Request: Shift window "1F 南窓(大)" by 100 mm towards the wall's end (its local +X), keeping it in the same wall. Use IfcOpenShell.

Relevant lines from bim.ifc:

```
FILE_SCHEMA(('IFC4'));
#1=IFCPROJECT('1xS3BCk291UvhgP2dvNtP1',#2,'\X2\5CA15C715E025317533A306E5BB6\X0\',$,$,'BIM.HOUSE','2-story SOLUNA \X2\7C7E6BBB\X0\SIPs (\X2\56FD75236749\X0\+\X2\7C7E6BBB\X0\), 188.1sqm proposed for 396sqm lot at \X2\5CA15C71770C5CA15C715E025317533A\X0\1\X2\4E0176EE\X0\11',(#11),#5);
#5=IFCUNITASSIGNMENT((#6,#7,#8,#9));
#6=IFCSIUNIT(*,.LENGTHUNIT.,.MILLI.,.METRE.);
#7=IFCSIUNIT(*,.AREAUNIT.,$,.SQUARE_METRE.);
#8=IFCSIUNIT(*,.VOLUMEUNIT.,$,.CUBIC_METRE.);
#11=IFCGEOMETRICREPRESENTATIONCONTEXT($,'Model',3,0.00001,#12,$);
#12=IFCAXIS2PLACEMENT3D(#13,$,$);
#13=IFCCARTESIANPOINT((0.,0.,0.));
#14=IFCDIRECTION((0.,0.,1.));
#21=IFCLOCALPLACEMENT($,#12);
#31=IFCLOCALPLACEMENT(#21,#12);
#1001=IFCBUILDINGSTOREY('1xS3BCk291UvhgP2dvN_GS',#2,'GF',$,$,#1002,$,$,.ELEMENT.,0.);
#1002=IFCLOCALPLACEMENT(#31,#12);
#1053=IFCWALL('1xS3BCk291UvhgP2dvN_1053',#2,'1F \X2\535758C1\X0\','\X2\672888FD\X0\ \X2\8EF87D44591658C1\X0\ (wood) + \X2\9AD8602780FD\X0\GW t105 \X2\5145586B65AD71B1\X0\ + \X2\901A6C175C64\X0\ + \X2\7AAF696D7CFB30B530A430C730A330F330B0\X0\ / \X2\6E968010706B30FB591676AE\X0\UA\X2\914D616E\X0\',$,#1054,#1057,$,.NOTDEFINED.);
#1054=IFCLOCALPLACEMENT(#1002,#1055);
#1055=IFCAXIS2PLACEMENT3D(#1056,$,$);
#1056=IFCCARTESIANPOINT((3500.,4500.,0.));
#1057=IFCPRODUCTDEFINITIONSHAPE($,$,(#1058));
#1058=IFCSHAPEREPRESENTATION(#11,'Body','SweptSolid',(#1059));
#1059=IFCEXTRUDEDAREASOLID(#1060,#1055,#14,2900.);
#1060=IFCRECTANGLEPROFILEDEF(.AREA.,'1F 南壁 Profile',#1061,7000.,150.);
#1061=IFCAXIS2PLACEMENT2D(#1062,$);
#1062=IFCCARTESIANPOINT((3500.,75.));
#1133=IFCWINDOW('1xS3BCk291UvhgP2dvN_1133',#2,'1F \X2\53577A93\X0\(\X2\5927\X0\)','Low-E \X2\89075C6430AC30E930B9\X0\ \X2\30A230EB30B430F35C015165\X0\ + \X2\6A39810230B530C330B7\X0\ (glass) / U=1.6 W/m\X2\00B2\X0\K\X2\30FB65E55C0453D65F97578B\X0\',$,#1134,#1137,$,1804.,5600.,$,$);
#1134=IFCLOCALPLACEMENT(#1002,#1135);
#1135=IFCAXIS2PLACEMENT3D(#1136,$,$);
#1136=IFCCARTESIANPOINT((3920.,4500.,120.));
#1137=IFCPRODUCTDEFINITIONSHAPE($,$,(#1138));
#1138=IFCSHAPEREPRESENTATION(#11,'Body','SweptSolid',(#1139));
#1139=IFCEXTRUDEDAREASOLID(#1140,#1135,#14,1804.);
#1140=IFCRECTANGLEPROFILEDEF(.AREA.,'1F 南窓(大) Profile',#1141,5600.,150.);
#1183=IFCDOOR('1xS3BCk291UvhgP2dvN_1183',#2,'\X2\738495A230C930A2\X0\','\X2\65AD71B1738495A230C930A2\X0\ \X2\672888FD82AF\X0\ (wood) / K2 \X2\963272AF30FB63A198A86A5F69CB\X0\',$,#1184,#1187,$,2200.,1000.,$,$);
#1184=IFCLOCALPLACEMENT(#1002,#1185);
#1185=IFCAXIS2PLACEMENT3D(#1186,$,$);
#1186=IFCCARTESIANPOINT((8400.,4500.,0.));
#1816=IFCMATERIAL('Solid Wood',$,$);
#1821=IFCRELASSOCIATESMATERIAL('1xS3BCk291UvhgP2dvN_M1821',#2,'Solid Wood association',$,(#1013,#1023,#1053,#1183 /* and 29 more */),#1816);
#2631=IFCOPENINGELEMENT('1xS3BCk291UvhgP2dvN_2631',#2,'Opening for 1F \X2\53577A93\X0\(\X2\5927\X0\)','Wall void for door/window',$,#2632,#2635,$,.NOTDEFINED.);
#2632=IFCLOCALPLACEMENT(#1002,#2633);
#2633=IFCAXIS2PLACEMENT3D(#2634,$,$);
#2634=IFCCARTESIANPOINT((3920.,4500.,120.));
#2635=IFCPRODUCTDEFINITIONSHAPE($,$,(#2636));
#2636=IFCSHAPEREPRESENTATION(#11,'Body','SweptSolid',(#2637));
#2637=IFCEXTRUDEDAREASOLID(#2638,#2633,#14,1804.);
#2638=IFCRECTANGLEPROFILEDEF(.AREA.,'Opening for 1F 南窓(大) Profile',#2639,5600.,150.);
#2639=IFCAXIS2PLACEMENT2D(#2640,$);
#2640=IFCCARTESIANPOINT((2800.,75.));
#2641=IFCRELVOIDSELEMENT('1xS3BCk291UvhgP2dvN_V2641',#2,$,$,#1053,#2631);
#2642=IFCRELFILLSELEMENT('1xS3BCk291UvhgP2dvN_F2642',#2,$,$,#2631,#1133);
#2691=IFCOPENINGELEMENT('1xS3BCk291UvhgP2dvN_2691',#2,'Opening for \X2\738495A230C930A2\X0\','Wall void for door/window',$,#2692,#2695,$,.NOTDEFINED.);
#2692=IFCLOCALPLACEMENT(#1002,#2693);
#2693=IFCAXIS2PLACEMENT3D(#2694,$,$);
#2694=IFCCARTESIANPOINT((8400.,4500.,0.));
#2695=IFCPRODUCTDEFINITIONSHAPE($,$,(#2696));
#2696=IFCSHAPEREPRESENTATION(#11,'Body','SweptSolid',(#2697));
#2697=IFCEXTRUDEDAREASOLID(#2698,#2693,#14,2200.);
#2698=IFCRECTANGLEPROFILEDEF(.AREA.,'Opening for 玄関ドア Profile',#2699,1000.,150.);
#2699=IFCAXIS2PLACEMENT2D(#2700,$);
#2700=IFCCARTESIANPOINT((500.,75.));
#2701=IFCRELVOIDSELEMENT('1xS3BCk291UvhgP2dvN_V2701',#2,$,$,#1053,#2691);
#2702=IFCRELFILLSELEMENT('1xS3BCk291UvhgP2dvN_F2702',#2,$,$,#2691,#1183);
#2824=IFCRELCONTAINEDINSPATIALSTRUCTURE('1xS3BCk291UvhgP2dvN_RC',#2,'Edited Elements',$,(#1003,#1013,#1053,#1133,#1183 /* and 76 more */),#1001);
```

```python
import ifcopenshell
import ifcopenshell.api.geometry
import ifcopenshell.util.placement

model = ifcopenshell.open("bim.ifc")

window = model.by_guid("1xS3BCk291UvhgP2dvN_1133")
opening = window.FillsVoids[0].RelatingOpeningElement
wall = opening.VoidsElements[0].RelatingBuildingElement

wall_matrix = ifcopenshell.util.placement.get_local_placement(wall.ObjectPlacement)
shift = wall_matrix[:3, 0] * 100.0
before = ifcopenshell.util.placement.get_local_placement(window.ObjectPlacement)[:3, 3].copy()

# The window is not placed relative to its opening, so move both.
for product in (opening, window):
    matrix = ifcopenshell.util.placement.get_local_placement(product.ObjectPlacement)
    matrix[:3, 3] += shift
    ifcopenshell.api.geometry.edit_object_placement(model, product=product, matrix=matrix, is_si=False)

after = ifcopenshell.util.placement.get_local_placement(window.ObjectPlacement)[:3, 3]
print("window moved by", (after - before).round(3) + 0.0)

model.write("bim-out.ifc")
```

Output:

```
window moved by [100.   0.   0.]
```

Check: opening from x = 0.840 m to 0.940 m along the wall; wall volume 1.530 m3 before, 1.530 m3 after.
